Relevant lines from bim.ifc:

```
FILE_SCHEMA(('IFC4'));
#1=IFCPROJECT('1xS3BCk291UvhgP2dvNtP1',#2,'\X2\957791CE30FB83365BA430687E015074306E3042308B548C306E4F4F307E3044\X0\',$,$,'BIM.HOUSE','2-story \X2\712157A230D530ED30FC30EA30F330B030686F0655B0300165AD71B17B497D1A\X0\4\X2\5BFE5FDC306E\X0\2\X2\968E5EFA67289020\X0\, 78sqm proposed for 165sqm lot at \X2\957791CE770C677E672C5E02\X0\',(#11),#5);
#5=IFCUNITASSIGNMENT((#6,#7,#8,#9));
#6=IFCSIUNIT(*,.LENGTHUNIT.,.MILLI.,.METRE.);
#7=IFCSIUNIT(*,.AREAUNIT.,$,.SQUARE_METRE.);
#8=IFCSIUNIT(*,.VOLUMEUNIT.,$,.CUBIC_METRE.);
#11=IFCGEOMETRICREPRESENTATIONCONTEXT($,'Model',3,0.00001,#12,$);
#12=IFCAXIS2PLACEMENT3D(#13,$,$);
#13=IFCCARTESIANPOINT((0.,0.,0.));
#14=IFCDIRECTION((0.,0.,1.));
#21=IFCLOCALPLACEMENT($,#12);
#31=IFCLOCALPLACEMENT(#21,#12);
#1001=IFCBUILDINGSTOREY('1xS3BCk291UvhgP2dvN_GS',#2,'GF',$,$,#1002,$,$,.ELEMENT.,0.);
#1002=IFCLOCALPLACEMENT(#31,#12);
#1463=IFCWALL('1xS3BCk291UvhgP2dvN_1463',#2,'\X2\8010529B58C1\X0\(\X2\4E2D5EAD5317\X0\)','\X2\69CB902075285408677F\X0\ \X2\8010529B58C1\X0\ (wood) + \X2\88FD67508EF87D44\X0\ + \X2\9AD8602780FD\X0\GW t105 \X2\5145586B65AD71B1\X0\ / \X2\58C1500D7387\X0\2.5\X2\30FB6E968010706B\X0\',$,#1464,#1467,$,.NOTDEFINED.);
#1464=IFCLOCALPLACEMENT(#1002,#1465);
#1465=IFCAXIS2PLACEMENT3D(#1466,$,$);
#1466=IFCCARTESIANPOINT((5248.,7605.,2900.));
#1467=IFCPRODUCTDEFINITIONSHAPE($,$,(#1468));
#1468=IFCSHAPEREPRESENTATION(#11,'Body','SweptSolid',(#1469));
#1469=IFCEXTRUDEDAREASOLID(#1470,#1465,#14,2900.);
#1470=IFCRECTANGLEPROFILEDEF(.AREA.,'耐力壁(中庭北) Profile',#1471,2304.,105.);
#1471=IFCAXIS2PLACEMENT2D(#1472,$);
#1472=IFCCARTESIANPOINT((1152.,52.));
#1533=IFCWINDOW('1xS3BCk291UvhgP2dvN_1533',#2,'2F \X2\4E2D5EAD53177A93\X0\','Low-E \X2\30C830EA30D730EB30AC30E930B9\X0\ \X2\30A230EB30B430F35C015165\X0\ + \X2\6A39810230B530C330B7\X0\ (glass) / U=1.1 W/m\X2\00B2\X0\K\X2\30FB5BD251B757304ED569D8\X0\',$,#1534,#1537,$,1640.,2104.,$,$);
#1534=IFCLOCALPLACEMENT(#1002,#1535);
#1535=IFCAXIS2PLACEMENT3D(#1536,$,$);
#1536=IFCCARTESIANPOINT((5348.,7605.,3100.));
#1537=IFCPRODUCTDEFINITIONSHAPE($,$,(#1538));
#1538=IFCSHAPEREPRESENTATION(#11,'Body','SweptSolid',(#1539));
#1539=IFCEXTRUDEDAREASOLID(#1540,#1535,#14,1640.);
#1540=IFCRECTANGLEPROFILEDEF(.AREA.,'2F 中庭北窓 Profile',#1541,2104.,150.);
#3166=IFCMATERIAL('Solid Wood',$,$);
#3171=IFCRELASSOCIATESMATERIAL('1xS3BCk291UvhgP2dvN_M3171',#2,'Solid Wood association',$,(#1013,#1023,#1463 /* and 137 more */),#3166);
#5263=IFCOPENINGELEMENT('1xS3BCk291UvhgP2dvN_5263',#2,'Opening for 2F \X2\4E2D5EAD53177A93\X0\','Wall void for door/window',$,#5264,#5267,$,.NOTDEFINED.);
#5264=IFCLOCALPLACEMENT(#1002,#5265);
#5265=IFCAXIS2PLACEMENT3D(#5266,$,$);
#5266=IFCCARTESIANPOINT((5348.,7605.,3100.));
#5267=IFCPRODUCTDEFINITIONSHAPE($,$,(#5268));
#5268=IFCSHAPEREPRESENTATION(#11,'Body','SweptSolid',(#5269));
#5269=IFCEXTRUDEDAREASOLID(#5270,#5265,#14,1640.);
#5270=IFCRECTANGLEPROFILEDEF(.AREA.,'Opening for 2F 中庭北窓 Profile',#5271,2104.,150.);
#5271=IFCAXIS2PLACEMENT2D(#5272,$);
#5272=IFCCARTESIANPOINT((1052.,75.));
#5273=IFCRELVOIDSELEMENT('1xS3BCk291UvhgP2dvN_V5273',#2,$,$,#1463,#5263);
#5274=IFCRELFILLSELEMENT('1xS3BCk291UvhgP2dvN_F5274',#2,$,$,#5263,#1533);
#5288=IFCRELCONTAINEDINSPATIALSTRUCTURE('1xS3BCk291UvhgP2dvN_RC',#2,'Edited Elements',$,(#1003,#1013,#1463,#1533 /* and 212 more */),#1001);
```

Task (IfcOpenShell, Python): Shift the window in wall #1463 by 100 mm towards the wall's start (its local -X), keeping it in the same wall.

```python
import ifcopenshell
import ifcopenshell.api.geometry
import ifcopenshell.util.placement

model = ifcopenshell.open("bim.ifc")

window = model.by_guid("1xS3BCk291UvhgP2dvN_1533")
opening = window.FillsVoids[0].RelatingOpeningElement
wall = opening.VoidsElements[0].RelatingBuildingElement

wall_matrix = ifcopenshell.util.placement.get_local_placement(wall.ObjectPlacement)
shift = wall_matrix[:3, 0] * -100.0
before = ifcopenshell.util.placement.get_local_placement(window.ObjectPlacement)[:3, 3].copy()

# The window is not placed relative to its opening, so move both.
for product in (opening, window):
    matrix = ifcopenshell.util.placement.get_local_placement(product.ObjectPlacement)
    matrix[:3, 3] += shift
    ifcopenshell.api.geometry.edit_object_placement(model, product=product, matrix=matrix, is_si=False)

after = ifcopenshell.util.placement.get_local_placement(window.ObjectPlacement)[:3, 3]
print("window moved by", (after - before).round(3) + 0.0)

model.write("bim_updated.ifc")
```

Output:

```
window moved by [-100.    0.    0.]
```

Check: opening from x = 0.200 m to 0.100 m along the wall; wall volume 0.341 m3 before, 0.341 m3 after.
